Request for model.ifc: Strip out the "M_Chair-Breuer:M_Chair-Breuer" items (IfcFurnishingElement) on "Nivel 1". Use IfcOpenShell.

First a look at what the model holds.

```python
import ifcopenshell
import ifcopenshell.util.element

model = ifcopenshell.open("model.ifc")
print(model.schema)
storey = next(s for s in model.by_type("IfcBuildingStorey") if s.Name == "Nivel 1")
furniture = [e for e in ifcopenshell.util.element.get_decomposition(storey) if e.is_a("IfcFurnishingElement")]
seen = {}
for e in furniture:
    element_type = ifcopenshell.util.element.get_type(e)
    name = element_type.Name if element_type not in (None, e) else None
    seen[name] = seen.get(name, 0) + 1
for name, count in sorted(seen.items(), key=str):
    print(count, "x", name)
```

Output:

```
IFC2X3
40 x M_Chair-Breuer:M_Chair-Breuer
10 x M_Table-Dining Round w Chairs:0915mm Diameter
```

```python
import ifcopenshell
import ifcopenshell.api.root
import ifcopenshell.util.element

model = ifcopenshell.open("model.ifc")

storey = next(s for s in model.by_type("IfcBuildingStorey") if s.Name == "Nivel 1")
furniture = [e for e in ifcopenshell.util.element.get_decomposition(storey) if e.is_a("IfcFurnishingElement")]
targets = [e for e in furniture if (t := ifcopenshell.util.element.get_type(e)) not in (None, e) and t.Name == "M_Chair-Breuer:M_Chair-Breuer"]

for e in targets:
    ifcopenshell.api.root.remove_product(model, product=e)
print(len(targets), "removed")

model.write("model_updated.ifc")
```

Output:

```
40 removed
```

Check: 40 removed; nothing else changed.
